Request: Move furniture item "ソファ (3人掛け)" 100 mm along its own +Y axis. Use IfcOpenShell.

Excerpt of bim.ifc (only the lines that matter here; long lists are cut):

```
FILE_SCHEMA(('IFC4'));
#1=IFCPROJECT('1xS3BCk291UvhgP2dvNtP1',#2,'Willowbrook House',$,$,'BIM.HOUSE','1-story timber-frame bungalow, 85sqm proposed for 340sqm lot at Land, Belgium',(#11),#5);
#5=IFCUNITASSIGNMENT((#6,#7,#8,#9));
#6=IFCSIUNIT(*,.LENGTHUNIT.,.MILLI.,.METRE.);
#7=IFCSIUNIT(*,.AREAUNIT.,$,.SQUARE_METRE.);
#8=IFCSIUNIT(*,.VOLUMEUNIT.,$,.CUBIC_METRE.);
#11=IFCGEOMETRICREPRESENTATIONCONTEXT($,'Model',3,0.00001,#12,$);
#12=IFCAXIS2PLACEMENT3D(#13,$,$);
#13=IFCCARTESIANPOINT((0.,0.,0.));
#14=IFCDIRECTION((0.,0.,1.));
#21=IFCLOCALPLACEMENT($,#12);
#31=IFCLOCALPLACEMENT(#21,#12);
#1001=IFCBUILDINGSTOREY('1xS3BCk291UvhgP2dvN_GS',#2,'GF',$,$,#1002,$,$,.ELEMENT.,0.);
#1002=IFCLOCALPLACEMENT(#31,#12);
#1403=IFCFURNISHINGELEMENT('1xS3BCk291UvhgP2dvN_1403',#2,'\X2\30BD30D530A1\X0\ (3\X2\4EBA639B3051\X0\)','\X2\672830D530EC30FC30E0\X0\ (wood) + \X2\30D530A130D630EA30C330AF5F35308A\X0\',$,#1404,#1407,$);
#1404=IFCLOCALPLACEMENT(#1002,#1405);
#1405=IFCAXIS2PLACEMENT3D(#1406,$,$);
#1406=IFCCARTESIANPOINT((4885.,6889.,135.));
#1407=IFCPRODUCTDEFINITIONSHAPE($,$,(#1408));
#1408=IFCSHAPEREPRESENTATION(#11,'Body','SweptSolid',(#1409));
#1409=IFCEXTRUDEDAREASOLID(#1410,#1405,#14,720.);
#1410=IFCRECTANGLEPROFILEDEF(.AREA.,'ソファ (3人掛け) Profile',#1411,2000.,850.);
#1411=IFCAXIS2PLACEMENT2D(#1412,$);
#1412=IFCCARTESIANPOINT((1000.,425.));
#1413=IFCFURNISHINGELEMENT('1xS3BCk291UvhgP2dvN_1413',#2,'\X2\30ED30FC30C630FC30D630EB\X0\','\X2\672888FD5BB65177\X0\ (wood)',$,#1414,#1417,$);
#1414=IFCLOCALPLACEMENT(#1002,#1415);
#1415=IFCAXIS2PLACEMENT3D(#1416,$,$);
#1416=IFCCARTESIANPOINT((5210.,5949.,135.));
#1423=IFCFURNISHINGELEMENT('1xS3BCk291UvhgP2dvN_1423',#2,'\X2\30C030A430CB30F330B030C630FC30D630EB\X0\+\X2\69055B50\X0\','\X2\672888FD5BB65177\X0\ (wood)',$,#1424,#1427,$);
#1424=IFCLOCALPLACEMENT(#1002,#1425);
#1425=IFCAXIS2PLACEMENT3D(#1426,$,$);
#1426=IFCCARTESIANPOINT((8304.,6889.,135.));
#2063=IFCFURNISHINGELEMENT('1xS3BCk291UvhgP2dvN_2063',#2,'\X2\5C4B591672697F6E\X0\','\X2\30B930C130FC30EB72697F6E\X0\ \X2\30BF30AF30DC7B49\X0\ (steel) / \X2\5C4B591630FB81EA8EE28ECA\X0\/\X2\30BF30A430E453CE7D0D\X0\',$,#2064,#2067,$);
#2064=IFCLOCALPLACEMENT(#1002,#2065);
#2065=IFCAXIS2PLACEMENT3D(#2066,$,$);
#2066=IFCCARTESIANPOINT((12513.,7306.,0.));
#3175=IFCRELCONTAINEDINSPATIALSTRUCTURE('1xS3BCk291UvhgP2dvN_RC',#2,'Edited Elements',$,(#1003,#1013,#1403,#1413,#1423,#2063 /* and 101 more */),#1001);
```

```python
import ifcopenshell
import ifcopenshell.api.geometry
import ifcopenshell.util.placement
import ifcopenshell.util.unit

model = ifcopenshell.open("bim.ifc")
unit_scale = ifcopenshell.util.unit.calculate_unit_scale(model)

item = model.by_guid("1xS3BCk291UvhgP2dvN_1403")
matrix = ifcopenshell.util.placement.get_local_placement(item.ObjectPlacement)
matrix[:3, 3] += matrix[:3, 1] * 0.1 / unit_scale
ifcopenshell.api.geometry.edit_object_placement(model, product=item, matrix=matrix, is_si=False)

print(ifcopenshell.util.placement.get_local_placement(item.ObjectPlacement).round(3) + 0.0)

model.write("bim_v2.ifc")
```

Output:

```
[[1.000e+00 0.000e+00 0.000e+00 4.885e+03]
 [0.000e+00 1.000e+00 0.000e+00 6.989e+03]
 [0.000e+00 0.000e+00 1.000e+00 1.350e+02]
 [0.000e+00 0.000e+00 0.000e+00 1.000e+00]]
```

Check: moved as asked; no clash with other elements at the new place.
